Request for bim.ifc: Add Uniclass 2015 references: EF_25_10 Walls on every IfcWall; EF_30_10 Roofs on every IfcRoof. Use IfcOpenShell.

First a look at what the model holds.

```python
import ifcopenshell

model = ifcopenshell.open("bim.ifc")
print(model.schema)
print("classifications:", [c.Name for c in model.by_type("IfcClassification")])
for ifc_class in ("IfcDoor", "IfcRoof", "IfcStair", "IfcWall", "IfcWindow"):
    print(ifc_class, len(model.by_type(ifc_class)))
```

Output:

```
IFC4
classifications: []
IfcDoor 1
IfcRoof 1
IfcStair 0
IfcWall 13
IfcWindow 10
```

```python
import ifcopenshell
import ifcopenshell.api.classification

model = ifcopenshell.open("bim.ifc")

system = ifcopenshell.api.classification.add_classification(model, classification="Uniclass 2015")

codes = {
    "IfcWall": ("EF_25_10", "Walls"),
    "IfcRoof": ("EF_30_10", "Roofs"),
}
for ifc_class, (code, name) in codes.items():
    products = model.by_type(ifc_class)
    ifcopenshell.api.classification.add_reference(
        model, products=products, classification=system, identification=code, name=name
    )
    print(code, len(products))

model.write("bim-out.ifc")
```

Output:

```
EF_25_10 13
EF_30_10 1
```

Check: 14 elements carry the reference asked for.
